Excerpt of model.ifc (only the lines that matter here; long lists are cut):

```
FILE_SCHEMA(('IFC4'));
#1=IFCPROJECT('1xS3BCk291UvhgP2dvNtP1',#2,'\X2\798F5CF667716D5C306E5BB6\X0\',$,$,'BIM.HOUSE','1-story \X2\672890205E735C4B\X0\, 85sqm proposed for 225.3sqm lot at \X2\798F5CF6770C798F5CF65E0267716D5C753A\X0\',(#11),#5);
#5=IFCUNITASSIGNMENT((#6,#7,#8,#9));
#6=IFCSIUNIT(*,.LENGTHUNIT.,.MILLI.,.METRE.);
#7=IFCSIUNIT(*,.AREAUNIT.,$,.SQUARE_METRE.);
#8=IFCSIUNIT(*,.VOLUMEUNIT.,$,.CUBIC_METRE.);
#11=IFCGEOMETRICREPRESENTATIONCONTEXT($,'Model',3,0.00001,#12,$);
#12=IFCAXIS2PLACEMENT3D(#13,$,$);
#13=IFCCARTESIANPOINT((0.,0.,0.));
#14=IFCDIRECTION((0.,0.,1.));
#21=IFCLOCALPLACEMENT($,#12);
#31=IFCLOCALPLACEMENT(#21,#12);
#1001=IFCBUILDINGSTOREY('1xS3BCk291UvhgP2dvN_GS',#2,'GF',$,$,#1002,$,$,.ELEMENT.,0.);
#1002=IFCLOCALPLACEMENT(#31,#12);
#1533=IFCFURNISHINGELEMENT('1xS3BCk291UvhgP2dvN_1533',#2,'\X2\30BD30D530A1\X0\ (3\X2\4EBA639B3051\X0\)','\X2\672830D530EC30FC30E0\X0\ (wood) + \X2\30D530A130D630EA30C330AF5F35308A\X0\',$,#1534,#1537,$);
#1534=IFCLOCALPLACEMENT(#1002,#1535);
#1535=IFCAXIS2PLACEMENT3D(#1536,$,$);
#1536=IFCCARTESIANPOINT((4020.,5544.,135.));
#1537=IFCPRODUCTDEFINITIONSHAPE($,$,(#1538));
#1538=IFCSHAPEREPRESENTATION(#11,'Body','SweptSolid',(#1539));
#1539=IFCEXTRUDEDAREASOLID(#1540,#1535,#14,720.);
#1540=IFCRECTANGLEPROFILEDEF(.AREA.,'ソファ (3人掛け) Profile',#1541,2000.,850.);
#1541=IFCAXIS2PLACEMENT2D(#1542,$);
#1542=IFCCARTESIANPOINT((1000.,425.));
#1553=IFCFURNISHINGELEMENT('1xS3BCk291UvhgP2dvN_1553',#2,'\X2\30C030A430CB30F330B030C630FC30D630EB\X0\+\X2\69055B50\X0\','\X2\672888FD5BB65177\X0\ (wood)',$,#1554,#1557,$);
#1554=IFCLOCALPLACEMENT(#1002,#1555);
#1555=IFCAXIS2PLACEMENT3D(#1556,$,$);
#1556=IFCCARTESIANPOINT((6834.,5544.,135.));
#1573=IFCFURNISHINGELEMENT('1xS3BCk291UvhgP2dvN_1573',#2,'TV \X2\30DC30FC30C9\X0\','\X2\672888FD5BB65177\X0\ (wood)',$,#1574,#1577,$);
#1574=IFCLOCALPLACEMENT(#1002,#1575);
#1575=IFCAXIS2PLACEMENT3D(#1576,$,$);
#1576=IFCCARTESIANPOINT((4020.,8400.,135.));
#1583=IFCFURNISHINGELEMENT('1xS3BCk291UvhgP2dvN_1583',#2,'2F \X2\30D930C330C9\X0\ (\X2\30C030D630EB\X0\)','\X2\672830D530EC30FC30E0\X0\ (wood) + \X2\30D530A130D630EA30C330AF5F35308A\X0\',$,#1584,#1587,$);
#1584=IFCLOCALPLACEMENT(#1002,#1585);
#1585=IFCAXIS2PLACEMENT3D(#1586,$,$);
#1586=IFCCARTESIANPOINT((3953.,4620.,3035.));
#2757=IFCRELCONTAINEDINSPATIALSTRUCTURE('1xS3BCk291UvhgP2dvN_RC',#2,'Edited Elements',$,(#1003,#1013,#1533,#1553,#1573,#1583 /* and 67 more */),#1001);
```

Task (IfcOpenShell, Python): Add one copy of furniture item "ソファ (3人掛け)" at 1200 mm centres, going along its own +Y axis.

```python
import ifcopenshell
import ifcopenshell.api.geometry
import ifcopenshell.api.root
import ifcopenshell.util.element
import ifcopenshell.util.placement
import ifcopenshell.util.unit

model = ifcopenshell.open("model.ifc")
unit_scale = ifcopenshell.util.unit.calculate_unit_scale(model)


def reuse_history(source, copy):
    """copy_class also copies each property set's owner history, people and application; keep the originals."""
    for rel in copy.IsDefinedBy:
        if rel.is_a("IfcRelDefinesByProperties") and (history := rel.RelatingPropertyDefinition.OwnerHistory):
            rel.RelatingPropertyDefinition.OwnerHistory = source.OwnerHistory
            ifcopenshell.util.element.remove_deep2(model, history)


source = model.by_guid("1xS3BCk291UvhgP2dvN_1533")
base = ifcopenshell.util.placement.get_local_placement(source.ObjectPlacement)
step = base[:3, 1] * 1.2 / unit_scale

for i in range(1, 2):
    copy = ifcopenshell.api.root.copy_class(model, product=source)
    copy.Representation = ifcopenshell.util.element.copy_deep(
        model, source.Representation, exclude=["IfcGeometricRepresentationContext", "IfcRepresentationMap"]
    )
    reuse_history(source, copy)
    matrix = base.copy()
    matrix[:3, 3] += i * step
    print("added at", matrix[:3, 3].round(3) + 0.0)
    ifcopenshell.api.geometry.edit_object_placement(model, product=copy, matrix=matrix, is_si=False)

model.write("model_v2.ifc")
```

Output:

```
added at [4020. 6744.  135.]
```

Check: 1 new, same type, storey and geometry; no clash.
